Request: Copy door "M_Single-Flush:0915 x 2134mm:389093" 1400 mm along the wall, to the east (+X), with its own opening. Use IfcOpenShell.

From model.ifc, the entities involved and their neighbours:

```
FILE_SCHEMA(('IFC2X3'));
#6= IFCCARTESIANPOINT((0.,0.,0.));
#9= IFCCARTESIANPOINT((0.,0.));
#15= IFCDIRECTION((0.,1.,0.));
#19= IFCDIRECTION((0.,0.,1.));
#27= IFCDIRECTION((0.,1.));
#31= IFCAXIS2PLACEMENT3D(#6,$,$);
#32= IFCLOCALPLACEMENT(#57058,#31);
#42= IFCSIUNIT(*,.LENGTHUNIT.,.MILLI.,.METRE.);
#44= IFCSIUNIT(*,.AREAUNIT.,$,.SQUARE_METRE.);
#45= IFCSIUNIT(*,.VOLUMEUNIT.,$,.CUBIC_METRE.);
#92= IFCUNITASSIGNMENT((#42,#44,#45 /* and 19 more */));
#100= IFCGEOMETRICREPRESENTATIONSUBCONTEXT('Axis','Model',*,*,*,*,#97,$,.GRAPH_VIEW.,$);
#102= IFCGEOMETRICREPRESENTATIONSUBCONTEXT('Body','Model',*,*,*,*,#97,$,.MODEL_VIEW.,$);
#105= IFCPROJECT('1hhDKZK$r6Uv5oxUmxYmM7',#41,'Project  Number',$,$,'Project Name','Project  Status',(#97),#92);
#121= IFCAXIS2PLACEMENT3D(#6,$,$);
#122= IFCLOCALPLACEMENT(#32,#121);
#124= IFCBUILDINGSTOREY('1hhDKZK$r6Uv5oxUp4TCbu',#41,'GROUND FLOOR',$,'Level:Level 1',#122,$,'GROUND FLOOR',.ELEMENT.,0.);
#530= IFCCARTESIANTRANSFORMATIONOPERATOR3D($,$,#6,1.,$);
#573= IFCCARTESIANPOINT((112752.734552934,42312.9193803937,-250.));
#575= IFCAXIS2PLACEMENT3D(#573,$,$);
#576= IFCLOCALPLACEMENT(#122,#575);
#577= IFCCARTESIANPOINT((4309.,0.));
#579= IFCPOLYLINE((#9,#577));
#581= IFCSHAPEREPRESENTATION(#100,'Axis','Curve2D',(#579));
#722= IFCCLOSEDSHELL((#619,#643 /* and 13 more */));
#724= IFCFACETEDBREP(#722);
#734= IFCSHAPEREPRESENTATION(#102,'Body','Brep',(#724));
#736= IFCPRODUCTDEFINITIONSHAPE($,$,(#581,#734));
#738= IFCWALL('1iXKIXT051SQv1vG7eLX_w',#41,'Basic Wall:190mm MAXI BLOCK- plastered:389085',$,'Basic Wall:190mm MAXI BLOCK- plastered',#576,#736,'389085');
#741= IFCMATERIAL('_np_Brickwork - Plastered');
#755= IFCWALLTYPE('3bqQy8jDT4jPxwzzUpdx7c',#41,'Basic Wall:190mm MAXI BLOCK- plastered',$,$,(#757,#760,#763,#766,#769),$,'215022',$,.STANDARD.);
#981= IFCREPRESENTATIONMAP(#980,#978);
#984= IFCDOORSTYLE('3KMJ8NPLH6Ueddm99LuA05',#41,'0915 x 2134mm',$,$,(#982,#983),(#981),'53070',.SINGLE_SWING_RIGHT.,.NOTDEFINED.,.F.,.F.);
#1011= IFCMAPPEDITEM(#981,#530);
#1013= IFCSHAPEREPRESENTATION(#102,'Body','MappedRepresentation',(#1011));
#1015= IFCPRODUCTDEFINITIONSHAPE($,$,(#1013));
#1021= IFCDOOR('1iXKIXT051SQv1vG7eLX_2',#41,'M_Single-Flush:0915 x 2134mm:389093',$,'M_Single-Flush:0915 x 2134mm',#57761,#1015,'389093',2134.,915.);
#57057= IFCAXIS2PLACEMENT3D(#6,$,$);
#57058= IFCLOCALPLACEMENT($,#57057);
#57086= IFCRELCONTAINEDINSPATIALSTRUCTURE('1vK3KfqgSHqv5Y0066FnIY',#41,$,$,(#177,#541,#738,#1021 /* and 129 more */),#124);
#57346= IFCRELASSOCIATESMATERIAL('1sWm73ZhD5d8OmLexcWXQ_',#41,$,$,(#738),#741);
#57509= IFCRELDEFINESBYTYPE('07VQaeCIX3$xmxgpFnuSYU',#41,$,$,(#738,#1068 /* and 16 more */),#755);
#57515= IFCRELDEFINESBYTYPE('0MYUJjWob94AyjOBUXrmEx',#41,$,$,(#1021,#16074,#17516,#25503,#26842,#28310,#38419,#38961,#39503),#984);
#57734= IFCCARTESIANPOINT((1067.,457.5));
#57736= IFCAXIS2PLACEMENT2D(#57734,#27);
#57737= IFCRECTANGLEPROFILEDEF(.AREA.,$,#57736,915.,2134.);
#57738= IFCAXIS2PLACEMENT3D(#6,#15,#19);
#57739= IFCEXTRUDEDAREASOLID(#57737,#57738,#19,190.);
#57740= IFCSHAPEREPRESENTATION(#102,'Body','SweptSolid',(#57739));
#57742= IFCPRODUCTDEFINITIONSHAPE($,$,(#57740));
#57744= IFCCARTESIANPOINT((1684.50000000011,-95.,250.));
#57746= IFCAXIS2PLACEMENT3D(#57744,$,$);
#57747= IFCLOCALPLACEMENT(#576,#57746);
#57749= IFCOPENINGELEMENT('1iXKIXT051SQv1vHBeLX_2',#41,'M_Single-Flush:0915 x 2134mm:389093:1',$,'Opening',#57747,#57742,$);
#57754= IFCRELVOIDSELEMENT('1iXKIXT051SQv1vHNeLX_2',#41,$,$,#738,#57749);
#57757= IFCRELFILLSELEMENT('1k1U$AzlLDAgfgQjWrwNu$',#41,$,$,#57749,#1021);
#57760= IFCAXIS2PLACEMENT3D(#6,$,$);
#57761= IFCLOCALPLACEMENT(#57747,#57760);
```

```python
import ifcopenshell
import ifcopenshell.api.feature
import ifcopenshell.api.geometry
import ifcopenshell.api.root
import ifcopenshell.geom
import ifcopenshell.util.element
import ifcopenshell.util.placement
import ifcopenshell.util.shape
import ifcopenshell.util.unit

model = ifcopenshell.open("model.ifc")
unit_scale = ifcopenshell.util.unit.calculate_unit_scale(model)
settings = ifcopenshell.geom.settings()


def volume(element):
    """Net volume in cubic metres, openings subtracted."""
    shape = ifcopenshell.geom.create_shape(settings, element)
    return ifcopenshell.util.shape.get_volume(shape.geometry)


def reuse_history(source, copy):
    """copy_class also copies each property set's owner history, people and application; keep the originals."""
    for rel in copy.IsDefinedBy:
        if rel.is_a("IfcRelDefinesByProperties") and (history := rel.RelatingPropertyDefinition.OwnerHistory):
            rel.RelatingPropertyDefinition.OwnerHistory = source.OwnerHistory
            ifcopenshell.util.element.remove_deep2(model, history)


door = model.by_guid("1iXKIXT051SQv1vG7eLX_2")
opening = door.FillsVoids[0].RelatingOpeningElement
wall = opening.VoidsElements[0].RelatingBuildingElement
before = volume(wall)
shift = ifcopenshell.util.placement.get_local_placement(wall.ObjectPlacement)[:3, 0] * 1.4 / unit_scale

# copy_class copies the void relationship, type, container and properties, but no geometry.
new_opening = ifcopenshell.api.root.copy_class(model, product=opening)
new_opening.Representation = ifcopenshell.util.element.copy_deep(
    model, opening.Representation, exclude=["IfcGeometricRepresentationContext", "IfcRepresentationMap"]
)
new_opening.Name = "M_Single-Flush:0915 x 2134mm"
new_door = ifcopenshell.api.root.copy_class(model, product=door)
new_door.Representation = ifcopenshell.util.element.copy_deep(
    model, door.Representation, exclude=["IfcGeometricRepresentationContext", "IfcRepresentationMap"]
)
new_door.Name = "M_Single-Flush:0915 x 2134mm"
new_door.Tag = None
reuse_history(door, new_door)
fills = ifcopenshell.api.feature.add_filling(model, opening=new_opening, element=new_door)
fills.OwnerHistory = new_door.OwnerHistory  # required in IFC2X3

for old, new in ((opening, new_opening), (door, new_door)):
    matrix = ifcopenshell.util.placement.get_local_placement(old.ObjectPlacement)
    matrix[:3, 3] += shift
    ifcopenshell.api.geometry.edit_object_placement(model, product=new, matrix=matrix, is_si=False)

after = volume(wall)

print(f"wall volume {before:.3f} -> {after:.3f} m3")

model.write("model_updated.ifc")
```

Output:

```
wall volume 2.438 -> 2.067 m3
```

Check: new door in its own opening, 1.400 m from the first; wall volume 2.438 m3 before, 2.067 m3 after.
